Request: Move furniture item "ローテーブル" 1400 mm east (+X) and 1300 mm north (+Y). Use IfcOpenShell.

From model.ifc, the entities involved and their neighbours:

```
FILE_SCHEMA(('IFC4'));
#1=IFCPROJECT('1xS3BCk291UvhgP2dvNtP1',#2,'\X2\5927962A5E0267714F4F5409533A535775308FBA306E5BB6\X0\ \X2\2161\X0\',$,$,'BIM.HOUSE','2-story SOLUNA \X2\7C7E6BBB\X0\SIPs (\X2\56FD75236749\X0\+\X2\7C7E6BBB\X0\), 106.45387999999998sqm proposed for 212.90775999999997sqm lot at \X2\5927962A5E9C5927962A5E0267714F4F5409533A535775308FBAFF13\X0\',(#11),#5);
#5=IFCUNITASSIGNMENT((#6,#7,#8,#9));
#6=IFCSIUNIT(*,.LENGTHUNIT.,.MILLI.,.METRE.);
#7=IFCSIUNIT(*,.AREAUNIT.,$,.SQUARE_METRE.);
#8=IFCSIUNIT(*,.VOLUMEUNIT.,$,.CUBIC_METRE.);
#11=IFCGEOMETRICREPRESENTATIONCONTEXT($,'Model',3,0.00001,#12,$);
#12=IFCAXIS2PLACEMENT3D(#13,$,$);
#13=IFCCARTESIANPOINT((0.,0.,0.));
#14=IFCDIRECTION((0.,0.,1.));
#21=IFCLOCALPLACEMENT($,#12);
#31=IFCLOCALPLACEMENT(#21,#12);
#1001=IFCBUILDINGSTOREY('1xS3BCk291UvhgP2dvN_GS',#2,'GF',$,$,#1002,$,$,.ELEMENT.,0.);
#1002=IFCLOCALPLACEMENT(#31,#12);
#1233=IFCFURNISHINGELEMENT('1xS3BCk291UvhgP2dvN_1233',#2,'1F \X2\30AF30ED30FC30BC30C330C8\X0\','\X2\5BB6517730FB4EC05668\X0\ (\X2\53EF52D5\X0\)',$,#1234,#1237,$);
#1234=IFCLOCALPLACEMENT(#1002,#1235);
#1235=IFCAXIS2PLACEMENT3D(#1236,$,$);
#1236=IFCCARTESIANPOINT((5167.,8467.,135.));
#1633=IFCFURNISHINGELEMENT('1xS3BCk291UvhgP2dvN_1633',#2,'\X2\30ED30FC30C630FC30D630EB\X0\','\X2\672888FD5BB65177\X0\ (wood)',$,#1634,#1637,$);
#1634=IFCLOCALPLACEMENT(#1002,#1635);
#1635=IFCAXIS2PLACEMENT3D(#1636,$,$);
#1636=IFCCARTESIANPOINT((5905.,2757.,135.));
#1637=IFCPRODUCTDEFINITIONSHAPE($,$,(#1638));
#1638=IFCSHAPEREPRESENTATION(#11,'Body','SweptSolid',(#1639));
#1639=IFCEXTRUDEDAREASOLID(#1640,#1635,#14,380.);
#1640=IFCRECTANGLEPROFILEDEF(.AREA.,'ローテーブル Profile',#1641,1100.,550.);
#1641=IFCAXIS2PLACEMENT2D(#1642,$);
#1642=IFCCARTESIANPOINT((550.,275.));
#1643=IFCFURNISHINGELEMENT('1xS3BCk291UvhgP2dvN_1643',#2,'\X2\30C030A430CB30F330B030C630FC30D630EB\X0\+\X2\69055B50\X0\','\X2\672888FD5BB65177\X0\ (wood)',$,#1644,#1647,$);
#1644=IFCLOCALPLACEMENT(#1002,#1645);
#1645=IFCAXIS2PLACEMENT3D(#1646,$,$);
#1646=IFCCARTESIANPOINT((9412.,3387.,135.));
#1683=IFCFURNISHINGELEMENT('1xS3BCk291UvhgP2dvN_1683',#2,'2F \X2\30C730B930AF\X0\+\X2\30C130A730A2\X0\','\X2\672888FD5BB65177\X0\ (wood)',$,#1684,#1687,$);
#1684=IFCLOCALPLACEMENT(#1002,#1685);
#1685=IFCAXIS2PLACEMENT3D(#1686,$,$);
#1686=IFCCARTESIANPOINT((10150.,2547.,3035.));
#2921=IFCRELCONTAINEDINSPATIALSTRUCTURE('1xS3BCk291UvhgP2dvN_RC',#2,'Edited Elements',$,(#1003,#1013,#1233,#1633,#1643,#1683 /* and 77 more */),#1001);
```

```python
import ifcopenshell
import ifcopenshell.api.geometry
import ifcopenshell.util.placement
import ifcopenshell.util.unit

model = ifcopenshell.open("model.ifc")
unit_scale = ifcopenshell.util.unit.calculate_unit_scale(model)

item = model.by_guid("1xS3BCk291UvhgP2dvN_1633")
matrix = ifcopenshell.util.placement.get_local_placement(item.ObjectPlacement)
matrix[0, 3] += 1.4 / unit_scale
matrix[1, 3] += 1.3 / unit_scale
ifcopenshell.api.geometry.edit_object_placement(model, product=item, matrix=matrix, is_si=False)

print(ifcopenshell.util.placement.get_local_placement(item.ObjectPlacement).round(3) + 0.0)

model.write("model-out.ifc")
```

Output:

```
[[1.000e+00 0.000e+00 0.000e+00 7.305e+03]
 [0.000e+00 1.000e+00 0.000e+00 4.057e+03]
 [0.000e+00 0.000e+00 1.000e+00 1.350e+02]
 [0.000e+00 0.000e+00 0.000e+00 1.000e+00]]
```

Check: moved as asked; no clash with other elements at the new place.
